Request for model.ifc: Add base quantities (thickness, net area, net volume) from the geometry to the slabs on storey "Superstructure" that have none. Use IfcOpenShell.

First a look at what the model holds.

```python
import ifcopenshell
import ifcopenshell.util.element
import ifcopenshell.util.unit

model = ifcopenshell.open("model.ifc")
print(model.schema)
for unit_type in ("LENGTHUNIT", "AREAUNIT", "VOLUMEUNIT"):
    print(unit_type, ifcopenshell.util.unit.calculate_unit_scale(model, unit_type))
storey = next(s for s in model.by_type("IfcBuildingStorey") if s.Name == "Superstructure")
slabs = [e for e in ifcopenshell.util.element.get_decomposition(storey) if e.is_a("IfcSlab")]
for e in sorted(slabs, key=lambda e: e.id()):
    print(e.id(), e.is_a(), e.Name, list(ifcopenshell.util.element.get_psets(e, qtos_only=True)), sep=" | ")
```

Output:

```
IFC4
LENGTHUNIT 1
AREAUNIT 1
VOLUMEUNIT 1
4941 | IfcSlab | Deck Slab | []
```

```python
import ifcopenshell
import ifcopenshell.api.pset
import ifcopenshell.geom
import ifcopenshell.util.element
import ifcopenshell.util.shape
import ifcopenshell.util.unit

model = ifcopenshell.open("model.ifc")
unit_scale = ifcopenshell.util.unit.calculate_unit_scale(model)
area_scale = ifcopenshell.util.unit.calculate_unit_scale(model, "AREAUNIT")
volume_scale = ifcopenshell.util.unit.calculate_unit_scale(model, "VOLUMEUNIT")
settings = ifcopenshell.geom.settings()

storey = next(s for s in model.by_type("IfcBuildingStorey") if s.Name == "Superstructure")
slabs = [e for e in ifcopenshell.util.element.get_decomposition(storey) if e.is_a("IfcSlab")]

for e in sorted(slabs, key=lambda e: e.id()):
    if ifcopenshell.util.element.get_psets(e, qtos_only=True, should_inherit=False):
        continue
    # Geometry comes back in metres, in the element's own axes.
    shape = ifcopenshell.geom.create_shape(settings, e)
    values = {
        "Width": ifcopenshell.util.shape.get_z(shape.geometry) / unit_scale,
        "NetArea": ifcopenshell.util.shape.get_footprint_area(shape.geometry) / area_scale,
        "NetVolume": ifcopenshell.util.shape.get_volume(shape.geometry) / volume_scale,
    }
    qto = ifcopenshell.api.pset.add_qto(model, product=e, name="Qto_SlabBaseQuantities")
    ifcopenshell.api.pset.edit_qto(model, qto=qto, properties=values)
    print(e.id(), {k: round(v, 3) for k, v in values.items()})

model.write("model_edited.ifc")
```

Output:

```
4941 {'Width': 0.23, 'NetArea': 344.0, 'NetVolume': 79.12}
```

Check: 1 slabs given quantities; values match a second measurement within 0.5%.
